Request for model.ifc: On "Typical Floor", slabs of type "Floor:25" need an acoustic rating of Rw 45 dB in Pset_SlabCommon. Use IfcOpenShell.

First a look at what the model holds.

```python
import ifcopenshell
import ifcopenshell.util.element

model = ifcopenshell.open("model.ifc")
print(model.schema)
storey = next(s for s in model.by_type("IfcBuildingStorey") if s.Name == "Typical Floor")
slabs = [e for e in ifcopenshell.util.element.get_decomposition(storey) if e.is_a("IfcSlab")]
seen = {}
for e in slabs:
    element_type = ifcopenshell.util.element.get_type(e)
    key = (element_type.Name if element_type != e and element_type else None, ifcopenshell.util.element.get_pset(e, "Pset_SlabCommon", "AcousticRating"))
    seen[key] = seen.get(key, 0) + 1
for (name, value), count in sorted(seen.items(), key=str):
    print(count, "x", name, "|", value)
```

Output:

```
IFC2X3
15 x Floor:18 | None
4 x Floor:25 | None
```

```python
import ifcopenshell
import ifcopenshell.api.pset
import ifcopenshell.util.element

model = ifcopenshell.open("model.ifc")

storey = next(s for s in model.by_type("IfcBuildingStorey") if s.Name == "Typical Floor")
slabs = [e for e in ifcopenshell.util.element.get_decomposition(storey) if e.is_a("IfcSlab")]

count = 0
for e in slabs:
    element_type = ifcopenshell.util.element.get_type(e)
    if element_type in (None, e) or element_type.Name != "Floor:25":
        continue
    # add_pset returns the element's existing set when there is one.
    pset = ifcopenshell.api.pset.add_pset(model, product=e, name="Pset_SlabCommon")
    ifcopenshell.api.pset.edit_pset(model, pset=pset, properties={"AcousticRating": "Rw 45 dB"})
    count += 1

print(count, "slabs updated")

model.write("model_updated.ifc")
```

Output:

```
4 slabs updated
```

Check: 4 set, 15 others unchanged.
